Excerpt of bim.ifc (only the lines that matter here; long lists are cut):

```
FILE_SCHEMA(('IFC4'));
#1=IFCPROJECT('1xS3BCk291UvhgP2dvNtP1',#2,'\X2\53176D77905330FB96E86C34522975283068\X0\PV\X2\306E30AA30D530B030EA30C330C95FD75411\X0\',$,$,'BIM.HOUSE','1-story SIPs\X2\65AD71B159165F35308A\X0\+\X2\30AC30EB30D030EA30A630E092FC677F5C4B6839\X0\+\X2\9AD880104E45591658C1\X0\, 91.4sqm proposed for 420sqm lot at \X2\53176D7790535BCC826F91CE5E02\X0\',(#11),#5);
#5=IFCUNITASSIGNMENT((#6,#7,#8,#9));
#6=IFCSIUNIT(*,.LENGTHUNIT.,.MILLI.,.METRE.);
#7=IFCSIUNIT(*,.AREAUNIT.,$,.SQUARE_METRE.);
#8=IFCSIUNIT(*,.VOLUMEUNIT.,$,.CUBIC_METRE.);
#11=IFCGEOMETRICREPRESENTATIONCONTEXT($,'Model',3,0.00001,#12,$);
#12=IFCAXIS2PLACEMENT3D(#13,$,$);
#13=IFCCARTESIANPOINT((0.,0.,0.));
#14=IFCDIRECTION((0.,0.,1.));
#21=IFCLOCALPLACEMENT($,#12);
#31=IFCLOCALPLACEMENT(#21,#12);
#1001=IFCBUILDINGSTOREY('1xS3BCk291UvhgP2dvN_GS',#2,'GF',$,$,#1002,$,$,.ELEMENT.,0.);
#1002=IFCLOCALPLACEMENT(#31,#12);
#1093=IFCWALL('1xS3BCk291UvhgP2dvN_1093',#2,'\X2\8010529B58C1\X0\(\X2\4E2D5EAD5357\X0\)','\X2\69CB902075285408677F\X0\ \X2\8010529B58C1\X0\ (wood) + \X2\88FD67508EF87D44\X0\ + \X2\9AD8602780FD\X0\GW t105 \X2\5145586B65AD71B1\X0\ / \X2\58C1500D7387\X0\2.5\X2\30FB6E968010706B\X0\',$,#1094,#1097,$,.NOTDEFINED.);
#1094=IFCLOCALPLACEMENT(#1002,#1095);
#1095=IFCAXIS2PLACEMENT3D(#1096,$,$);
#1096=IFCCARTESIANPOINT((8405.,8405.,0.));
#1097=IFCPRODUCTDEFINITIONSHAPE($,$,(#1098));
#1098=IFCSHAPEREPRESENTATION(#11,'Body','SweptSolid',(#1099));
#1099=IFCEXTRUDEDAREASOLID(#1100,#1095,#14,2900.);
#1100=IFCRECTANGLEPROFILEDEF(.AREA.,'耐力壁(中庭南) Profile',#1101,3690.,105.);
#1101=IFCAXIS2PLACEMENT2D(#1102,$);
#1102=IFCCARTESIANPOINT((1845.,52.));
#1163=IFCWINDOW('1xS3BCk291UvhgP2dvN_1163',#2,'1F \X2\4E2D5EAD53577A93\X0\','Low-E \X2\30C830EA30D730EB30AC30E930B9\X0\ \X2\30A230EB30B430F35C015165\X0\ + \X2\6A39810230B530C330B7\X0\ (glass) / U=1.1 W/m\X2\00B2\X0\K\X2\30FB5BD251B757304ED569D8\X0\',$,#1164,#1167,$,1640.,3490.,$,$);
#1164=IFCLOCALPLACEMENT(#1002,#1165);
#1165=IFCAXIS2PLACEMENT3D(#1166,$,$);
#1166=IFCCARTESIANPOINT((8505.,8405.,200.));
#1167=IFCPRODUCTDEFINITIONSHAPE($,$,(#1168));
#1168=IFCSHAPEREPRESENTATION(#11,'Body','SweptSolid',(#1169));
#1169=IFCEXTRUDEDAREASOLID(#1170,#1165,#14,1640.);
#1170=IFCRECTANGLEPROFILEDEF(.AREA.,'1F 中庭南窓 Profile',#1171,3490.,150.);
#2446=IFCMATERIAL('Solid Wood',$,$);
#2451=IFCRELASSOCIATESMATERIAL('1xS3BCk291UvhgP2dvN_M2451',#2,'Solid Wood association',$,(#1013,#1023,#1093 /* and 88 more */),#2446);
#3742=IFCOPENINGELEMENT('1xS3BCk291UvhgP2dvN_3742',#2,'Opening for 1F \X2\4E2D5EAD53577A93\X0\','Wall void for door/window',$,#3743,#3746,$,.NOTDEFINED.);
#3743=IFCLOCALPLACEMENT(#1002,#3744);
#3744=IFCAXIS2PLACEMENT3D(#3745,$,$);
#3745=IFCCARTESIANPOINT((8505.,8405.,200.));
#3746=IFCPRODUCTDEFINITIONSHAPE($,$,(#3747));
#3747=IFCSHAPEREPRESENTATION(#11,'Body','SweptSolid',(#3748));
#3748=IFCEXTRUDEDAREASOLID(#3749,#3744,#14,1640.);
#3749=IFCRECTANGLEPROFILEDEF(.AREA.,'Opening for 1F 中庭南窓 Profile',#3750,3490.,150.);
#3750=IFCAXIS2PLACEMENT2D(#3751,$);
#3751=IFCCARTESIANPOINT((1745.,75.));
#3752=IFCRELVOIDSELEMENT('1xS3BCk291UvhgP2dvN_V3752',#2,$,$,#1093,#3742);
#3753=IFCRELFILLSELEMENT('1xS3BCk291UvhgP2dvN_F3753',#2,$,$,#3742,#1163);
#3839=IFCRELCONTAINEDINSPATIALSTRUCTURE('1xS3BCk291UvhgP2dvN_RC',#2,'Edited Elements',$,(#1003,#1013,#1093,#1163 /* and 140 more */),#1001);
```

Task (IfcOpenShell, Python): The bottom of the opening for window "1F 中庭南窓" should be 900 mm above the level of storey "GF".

```python
import numpy as np
import ifcopenshell
import ifcopenshell.api.geometry
import ifcopenshell.geom
import ifcopenshell.util.element
import ifcopenshell.util.placement
import ifcopenshell.util.shape
import ifcopenshell.util.unit

model = ifcopenshell.open("bim.ifc")
unit_scale = ifcopenshell.util.unit.calculate_unit_scale(model)

window = model.by_guid("1xS3BCk291UvhgP2dvN_1163")
opening = window.FillsVoids[0].RelatingOpeningElement
storey = ifcopenshell.util.element.get_container(window, ifc_class="IfcBuildingStorey")
level = ifcopenshell.util.placement.get_local_placement(storey.ObjectPlacement)[2, 3]

# The opening's origin need not be at the sill, so measure its lowest point.
shape = ifcopenshell.geom.create_shape(ifcopenshell.geom.settings(), opening)
bottom = ifcopenshell.util.shape.get_shape_bottom_elevation(shape, shape.geometry) / unit_scale
dz = level + 0.9 / unit_scale - bottom

shift = np.array([0.0, 0.0, dz])
# The window is not placed relative to its opening, so move both.
for product in (opening, window):
    matrix = ifcopenshell.util.placement.get_local_placement(product.ObjectPlacement)
    matrix[:3, 3] += shift
    ifcopenshell.api.geometry.edit_object_placement(model, product=product, matrix=matrix, is_si=False)

print(f"moved by {dz * unit_scale:+.3f} m")

model.write("bim_edited.ifc")
```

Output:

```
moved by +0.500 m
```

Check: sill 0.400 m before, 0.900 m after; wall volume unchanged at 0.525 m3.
